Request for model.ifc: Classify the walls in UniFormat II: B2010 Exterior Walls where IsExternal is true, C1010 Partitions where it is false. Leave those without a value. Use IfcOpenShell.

First a look at what the model holds.

```python
import ifcopenshell
import ifcopenshell.util.element

model = ifcopenshell.open("model.ifc")
print(model.schema)
print("classifications:", [c.Name for c in model.by_type("IfcClassification")])
values = [ifcopenshell.util.element.get_pset(e, "Pset_WallCommon", "IsExternal") for e in model.by_type("IfcWall")]
for value in (True, False, None):
    print("IsExternal", value, values.count(value))
```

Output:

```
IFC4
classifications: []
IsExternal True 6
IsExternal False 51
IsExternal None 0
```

```python
import ifcopenshell
import ifcopenshell.api.classification
import ifcopenshell.util.element

model = ifcopenshell.open("model.ifc")

system = ifcopenshell.api.classification.add_classification(model, classification="UniFormat II")

walls = model.by_type("IfcWall")
external = {e: ifcopenshell.util.element.get_pset(e, "Pset_WallCommon", "IsExternal") for e in walls}
for flag, code, name in ((True, "B2010", "Exterior Walls"), (False, "C1010", "Partitions")):
    products = [e for e in walls if external[e] is flag]
    ifcopenshell.api.classification.add_reference(
        model, products=products, classification=system, identification=code, name=name
    )
    print(code, len(products))

model.write("model_updated.ifc")
```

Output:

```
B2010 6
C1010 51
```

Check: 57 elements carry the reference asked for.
